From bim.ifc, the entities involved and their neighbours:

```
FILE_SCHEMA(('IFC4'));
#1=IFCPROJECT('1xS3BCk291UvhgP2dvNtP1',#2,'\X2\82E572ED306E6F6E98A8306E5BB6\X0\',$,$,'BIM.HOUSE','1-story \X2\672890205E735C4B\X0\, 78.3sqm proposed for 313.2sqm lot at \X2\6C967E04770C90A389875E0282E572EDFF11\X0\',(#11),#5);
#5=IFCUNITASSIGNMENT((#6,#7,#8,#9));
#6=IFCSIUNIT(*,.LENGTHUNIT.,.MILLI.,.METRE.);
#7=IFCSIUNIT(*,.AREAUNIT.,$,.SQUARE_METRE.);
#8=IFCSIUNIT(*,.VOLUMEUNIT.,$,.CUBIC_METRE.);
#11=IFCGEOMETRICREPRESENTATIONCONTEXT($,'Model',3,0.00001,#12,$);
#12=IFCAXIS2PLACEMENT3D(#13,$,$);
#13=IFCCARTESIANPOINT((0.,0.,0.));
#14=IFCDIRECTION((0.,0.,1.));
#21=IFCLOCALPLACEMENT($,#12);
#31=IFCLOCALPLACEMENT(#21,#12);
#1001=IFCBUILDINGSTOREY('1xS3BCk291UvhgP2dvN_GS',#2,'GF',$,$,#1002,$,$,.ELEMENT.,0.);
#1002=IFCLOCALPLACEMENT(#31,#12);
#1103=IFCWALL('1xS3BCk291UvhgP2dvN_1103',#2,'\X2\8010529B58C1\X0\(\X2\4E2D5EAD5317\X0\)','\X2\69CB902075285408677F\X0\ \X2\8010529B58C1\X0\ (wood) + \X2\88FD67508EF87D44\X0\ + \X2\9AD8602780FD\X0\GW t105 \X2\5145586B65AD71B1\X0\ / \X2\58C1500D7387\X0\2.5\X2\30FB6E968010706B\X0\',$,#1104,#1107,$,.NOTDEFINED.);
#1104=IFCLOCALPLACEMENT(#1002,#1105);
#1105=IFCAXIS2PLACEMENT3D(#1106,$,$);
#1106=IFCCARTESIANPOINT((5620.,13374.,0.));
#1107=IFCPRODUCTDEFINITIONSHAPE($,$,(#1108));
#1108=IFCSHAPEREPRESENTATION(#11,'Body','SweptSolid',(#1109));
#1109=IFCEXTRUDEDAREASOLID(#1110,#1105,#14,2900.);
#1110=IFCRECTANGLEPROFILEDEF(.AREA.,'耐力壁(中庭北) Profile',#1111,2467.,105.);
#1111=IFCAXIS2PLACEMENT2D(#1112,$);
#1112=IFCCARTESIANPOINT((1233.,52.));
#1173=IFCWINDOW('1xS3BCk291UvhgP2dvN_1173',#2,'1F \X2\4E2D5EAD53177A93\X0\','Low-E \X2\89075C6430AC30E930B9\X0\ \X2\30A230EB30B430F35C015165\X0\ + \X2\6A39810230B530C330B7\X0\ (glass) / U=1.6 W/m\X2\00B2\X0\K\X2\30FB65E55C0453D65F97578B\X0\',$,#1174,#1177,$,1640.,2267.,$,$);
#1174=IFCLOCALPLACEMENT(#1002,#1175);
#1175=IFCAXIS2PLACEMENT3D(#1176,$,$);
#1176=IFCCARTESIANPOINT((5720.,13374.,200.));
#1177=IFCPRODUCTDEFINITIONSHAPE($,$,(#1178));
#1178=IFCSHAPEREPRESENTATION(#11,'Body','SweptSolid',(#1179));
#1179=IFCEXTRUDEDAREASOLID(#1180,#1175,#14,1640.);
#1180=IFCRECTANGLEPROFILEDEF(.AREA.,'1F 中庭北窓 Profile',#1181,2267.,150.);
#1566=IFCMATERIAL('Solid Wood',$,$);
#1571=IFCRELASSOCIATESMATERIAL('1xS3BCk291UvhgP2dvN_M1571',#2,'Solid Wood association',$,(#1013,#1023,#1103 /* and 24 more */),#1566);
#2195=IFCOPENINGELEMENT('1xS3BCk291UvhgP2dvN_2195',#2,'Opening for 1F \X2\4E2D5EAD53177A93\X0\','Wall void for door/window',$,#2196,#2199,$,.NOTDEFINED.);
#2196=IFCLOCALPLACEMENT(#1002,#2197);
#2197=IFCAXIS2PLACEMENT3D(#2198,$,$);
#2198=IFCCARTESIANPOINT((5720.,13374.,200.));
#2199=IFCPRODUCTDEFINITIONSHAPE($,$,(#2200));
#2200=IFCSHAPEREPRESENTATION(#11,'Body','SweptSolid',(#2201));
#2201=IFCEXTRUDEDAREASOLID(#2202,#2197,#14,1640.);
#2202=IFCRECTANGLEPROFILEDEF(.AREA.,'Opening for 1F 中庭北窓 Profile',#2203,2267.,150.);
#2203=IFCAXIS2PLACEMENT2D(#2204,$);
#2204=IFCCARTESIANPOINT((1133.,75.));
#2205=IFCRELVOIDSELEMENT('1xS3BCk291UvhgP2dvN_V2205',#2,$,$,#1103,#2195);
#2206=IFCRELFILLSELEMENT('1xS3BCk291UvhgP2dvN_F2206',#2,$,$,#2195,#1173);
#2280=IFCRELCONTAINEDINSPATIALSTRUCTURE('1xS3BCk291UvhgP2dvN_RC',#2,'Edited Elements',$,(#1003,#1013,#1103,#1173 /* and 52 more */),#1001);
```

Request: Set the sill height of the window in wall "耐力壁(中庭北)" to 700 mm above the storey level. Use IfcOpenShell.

```python
import numpy as np
import ifcopenshell
import ifcopenshell.api.geometry
import ifcopenshell.geom
import ifcopenshell.util.element
import ifcopenshell.util.placement
import ifcopenshell.util.shape
import ifcopenshell.util.unit

model = ifcopenshell.open("bim.ifc")
unit_scale = ifcopenshell.util.unit.calculate_unit_scale(model)

window = model.by_guid("1xS3BCk291UvhgP2dvN_1173")
opening = window.FillsVoids[0].RelatingOpeningElement
storey = ifcopenshell.util.element.get_container(window, ifc_class="IfcBuildingStorey")
level = ifcopenshell.util.placement.get_local_placement(storey.ObjectPlacement)[2, 3]

# The opening's origin need not be at the sill, so measure its lowest point.
shape = ifcopenshell.geom.create_shape(ifcopenshell.geom.settings(), opening)
bottom = ifcopenshell.util.shape.get_shape_bottom_elevation(shape, shape.geometry) / unit_scale
dz = level + 0.7 / unit_scale - bottom

shift = np.array([0.0, 0.0, dz])
# The window is not placed relative to its opening, so move both.
for product in (opening, window):
    matrix = ifcopenshell.util.placement.get_local_placement(product.ObjectPlacement)
    matrix[:3, 3] += shift
    ifcopenshell.api.geometry.edit_object_placement(model, product=product, matrix=matrix, is_si=False)

print(f"moved by {dz * unit_scale:+.3f} m")

model.write("bim_v2.ifc")
```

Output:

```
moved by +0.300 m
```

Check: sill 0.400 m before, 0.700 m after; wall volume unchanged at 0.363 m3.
